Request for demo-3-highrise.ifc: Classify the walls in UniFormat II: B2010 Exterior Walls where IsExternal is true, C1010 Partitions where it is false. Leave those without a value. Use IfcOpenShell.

First a look at what the model holds.

```python
import ifcopenshell
import ifcopenshell.util.element

model = ifcopenshell.open("demo-3-highrise.ifc")
print(model.schema)
print("classifications:", [c.Name for c in model.by_type("IfcClassification")])
values = [ifcopenshell.util.element.get_pset(e, "Pset_WallCommon", "IsExternal") for e in model.by_type("IfcWall")]
for value in (True, False, None):
    print("IsExternal", value, values.count(value))
```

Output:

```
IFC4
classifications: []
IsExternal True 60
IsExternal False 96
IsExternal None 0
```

```python
import ifcopenshell
import ifcopenshell.api.classification
import ifcopenshell.util.element

model = ifcopenshell.open("demo-3-highrise.ifc")

system = ifcopenshell.api.classification.add_classification(model, classification="UniFormat II")

walls = model.by_type("IfcWall")
external = {e: ifcopenshell.util.element.get_pset(e, "Pset_WallCommon", "IsExternal") for e in walls}
for flag, code, name in ((True, "B2010", "Exterior Walls"), (False, "C1010", "Partitions")):
    products = [e for e in walls if external[e] is flag]
    ifcopenshell.api.classification.add_reference(
        model, products=products, classification=system, identification=code, name=name
    )
    print(code, len(products))

model.write("demo-3-highrise_updated.ifc")
```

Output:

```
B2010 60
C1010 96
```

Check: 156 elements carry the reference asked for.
